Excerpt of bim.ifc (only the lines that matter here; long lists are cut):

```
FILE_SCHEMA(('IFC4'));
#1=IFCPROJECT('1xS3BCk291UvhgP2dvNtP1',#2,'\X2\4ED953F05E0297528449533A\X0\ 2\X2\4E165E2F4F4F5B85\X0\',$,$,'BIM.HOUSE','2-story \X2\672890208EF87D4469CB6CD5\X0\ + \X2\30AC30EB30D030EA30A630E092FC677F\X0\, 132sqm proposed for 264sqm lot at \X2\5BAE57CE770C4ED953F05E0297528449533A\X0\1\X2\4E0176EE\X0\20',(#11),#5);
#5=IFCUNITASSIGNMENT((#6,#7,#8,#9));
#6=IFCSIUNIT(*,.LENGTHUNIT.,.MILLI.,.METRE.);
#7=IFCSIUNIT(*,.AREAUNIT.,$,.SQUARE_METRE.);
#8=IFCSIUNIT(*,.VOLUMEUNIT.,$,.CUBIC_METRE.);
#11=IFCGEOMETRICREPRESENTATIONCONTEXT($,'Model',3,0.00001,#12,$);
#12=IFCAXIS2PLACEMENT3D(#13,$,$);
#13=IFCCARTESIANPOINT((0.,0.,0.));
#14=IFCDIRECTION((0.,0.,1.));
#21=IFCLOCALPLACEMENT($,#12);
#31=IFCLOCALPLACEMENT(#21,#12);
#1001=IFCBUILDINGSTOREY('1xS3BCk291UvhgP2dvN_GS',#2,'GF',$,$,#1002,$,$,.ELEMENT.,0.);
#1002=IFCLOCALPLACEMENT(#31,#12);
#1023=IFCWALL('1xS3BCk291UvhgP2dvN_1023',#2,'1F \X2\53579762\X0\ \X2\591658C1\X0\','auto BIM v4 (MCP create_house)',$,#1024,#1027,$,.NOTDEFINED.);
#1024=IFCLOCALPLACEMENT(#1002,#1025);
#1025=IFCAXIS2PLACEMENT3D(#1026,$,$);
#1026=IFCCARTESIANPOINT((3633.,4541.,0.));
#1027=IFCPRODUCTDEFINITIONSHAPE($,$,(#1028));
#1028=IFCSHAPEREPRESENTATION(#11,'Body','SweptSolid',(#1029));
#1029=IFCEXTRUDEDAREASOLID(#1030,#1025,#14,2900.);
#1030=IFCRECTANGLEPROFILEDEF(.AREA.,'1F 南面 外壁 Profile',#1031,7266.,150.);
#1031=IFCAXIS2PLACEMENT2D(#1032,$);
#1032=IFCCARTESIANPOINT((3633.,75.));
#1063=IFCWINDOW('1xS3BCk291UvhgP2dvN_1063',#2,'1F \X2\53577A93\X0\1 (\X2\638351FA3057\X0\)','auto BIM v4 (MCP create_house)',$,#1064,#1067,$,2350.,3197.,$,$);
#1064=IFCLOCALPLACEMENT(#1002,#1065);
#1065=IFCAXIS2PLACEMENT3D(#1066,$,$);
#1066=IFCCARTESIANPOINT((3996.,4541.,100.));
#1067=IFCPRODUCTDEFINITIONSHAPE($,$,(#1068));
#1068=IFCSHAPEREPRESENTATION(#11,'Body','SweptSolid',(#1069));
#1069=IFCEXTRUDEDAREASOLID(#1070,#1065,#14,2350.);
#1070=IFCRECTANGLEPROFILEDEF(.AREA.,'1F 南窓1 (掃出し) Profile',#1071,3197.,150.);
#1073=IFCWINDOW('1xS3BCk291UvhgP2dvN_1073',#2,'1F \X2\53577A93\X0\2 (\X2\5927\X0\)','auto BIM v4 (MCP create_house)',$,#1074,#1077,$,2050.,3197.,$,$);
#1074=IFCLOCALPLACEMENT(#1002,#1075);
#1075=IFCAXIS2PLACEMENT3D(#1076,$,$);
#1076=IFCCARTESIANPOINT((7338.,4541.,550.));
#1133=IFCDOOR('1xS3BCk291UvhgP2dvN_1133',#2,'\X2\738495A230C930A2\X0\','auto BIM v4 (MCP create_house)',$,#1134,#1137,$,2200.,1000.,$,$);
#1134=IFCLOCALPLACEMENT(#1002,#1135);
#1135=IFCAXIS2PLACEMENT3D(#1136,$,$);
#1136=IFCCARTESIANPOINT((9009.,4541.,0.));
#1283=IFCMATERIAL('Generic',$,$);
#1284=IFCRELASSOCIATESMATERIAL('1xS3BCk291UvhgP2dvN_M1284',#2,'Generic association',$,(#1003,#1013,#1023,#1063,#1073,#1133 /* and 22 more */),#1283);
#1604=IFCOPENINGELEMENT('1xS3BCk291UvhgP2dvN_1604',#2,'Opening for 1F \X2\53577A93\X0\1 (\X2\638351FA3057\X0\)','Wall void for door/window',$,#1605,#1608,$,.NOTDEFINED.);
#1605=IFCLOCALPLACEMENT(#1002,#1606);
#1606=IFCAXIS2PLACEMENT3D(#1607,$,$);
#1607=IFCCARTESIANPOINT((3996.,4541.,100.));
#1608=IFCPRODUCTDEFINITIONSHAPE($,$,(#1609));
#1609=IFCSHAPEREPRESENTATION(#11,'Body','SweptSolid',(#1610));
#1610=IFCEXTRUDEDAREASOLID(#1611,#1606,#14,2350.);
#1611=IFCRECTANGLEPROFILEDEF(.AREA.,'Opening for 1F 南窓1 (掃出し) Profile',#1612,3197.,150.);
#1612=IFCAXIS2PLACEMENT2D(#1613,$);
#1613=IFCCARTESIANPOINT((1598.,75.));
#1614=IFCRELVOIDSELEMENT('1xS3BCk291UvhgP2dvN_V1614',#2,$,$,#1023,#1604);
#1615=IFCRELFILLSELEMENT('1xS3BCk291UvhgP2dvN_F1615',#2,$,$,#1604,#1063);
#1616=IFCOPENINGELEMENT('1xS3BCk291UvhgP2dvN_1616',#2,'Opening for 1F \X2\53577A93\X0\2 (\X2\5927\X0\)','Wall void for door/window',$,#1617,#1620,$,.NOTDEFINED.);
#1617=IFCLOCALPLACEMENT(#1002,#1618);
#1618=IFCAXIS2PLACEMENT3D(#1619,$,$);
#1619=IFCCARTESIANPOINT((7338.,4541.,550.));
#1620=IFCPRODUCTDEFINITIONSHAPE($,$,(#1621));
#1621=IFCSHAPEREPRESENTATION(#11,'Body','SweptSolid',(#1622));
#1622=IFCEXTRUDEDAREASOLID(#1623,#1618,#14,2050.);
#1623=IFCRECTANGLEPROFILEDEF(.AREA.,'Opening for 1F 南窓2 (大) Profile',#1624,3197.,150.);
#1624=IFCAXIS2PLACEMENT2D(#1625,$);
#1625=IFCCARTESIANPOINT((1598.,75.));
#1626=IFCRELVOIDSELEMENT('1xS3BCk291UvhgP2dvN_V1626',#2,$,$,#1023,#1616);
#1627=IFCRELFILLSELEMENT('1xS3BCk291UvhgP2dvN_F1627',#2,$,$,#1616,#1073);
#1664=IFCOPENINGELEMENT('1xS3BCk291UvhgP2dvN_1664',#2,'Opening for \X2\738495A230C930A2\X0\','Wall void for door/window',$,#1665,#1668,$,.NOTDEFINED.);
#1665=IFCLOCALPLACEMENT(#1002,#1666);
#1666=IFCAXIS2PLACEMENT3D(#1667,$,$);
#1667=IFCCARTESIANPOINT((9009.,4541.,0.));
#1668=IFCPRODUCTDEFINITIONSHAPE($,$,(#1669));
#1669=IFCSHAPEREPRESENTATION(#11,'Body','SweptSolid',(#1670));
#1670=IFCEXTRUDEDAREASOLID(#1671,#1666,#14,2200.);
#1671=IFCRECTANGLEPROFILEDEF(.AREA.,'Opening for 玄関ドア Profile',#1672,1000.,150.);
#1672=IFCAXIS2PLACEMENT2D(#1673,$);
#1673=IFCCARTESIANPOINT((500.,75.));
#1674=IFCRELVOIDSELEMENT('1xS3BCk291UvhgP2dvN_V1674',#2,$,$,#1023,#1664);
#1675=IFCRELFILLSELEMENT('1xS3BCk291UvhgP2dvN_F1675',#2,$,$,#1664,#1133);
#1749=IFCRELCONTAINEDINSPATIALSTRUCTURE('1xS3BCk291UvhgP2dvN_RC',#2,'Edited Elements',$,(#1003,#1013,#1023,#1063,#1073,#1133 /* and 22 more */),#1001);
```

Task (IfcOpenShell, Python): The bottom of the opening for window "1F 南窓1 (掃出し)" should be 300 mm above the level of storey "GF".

```python
import numpy as np
import ifcopenshell
import ifcopenshell.api.geometry
import ifcopenshell.geom
import ifcopenshell.util.element
import ifcopenshell.util.placement
import ifcopenshell.util.shape
import ifcopenshell.util.unit

model = ifcopenshell.open("bim.ifc")
unit_scale = ifcopenshell.util.unit.calculate_unit_scale(model)

window = model.by_guid("1xS3BCk291UvhgP2dvN_1063")
opening = window.FillsVoids[0].RelatingOpeningElement
storey = ifcopenshell.util.element.get_container(window, ifc_class="IfcBuildingStorey")
level = ifcopenshell.util.placement.get_local_placement(storey.ObjectPlacement)[2, 3]

# The opening's origin need not be at the sill, so measure its lowest point.
shape = ifcopenshell.geom.create_shape(ifcopenshell.geom.settings(), opening)
bottom = ifcopenshell.util.shape.get_shape_bottom_elevation(shape, shape.geometry) / unit_scale
dz = level + 300.0 - bottom

shift = np.array([0.0, 0.0, dz])
# The window is not placed relative to its opening, so move both.
for product in (opening, window):
    matrix = ifcopenshell.util.placement.get_local_placement(product.ObjectPlacement)
    matrix[:3, 3] += shift
    ifcopenshell.api.geometry.edit_object_placement(model, product=product, matrix=matrix, is_si=False)

print(f"moved by {dz * unit_scale:+.3f} m")

model.write("bim_edited.ifc")
```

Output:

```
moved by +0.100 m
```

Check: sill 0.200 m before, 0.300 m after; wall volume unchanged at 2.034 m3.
